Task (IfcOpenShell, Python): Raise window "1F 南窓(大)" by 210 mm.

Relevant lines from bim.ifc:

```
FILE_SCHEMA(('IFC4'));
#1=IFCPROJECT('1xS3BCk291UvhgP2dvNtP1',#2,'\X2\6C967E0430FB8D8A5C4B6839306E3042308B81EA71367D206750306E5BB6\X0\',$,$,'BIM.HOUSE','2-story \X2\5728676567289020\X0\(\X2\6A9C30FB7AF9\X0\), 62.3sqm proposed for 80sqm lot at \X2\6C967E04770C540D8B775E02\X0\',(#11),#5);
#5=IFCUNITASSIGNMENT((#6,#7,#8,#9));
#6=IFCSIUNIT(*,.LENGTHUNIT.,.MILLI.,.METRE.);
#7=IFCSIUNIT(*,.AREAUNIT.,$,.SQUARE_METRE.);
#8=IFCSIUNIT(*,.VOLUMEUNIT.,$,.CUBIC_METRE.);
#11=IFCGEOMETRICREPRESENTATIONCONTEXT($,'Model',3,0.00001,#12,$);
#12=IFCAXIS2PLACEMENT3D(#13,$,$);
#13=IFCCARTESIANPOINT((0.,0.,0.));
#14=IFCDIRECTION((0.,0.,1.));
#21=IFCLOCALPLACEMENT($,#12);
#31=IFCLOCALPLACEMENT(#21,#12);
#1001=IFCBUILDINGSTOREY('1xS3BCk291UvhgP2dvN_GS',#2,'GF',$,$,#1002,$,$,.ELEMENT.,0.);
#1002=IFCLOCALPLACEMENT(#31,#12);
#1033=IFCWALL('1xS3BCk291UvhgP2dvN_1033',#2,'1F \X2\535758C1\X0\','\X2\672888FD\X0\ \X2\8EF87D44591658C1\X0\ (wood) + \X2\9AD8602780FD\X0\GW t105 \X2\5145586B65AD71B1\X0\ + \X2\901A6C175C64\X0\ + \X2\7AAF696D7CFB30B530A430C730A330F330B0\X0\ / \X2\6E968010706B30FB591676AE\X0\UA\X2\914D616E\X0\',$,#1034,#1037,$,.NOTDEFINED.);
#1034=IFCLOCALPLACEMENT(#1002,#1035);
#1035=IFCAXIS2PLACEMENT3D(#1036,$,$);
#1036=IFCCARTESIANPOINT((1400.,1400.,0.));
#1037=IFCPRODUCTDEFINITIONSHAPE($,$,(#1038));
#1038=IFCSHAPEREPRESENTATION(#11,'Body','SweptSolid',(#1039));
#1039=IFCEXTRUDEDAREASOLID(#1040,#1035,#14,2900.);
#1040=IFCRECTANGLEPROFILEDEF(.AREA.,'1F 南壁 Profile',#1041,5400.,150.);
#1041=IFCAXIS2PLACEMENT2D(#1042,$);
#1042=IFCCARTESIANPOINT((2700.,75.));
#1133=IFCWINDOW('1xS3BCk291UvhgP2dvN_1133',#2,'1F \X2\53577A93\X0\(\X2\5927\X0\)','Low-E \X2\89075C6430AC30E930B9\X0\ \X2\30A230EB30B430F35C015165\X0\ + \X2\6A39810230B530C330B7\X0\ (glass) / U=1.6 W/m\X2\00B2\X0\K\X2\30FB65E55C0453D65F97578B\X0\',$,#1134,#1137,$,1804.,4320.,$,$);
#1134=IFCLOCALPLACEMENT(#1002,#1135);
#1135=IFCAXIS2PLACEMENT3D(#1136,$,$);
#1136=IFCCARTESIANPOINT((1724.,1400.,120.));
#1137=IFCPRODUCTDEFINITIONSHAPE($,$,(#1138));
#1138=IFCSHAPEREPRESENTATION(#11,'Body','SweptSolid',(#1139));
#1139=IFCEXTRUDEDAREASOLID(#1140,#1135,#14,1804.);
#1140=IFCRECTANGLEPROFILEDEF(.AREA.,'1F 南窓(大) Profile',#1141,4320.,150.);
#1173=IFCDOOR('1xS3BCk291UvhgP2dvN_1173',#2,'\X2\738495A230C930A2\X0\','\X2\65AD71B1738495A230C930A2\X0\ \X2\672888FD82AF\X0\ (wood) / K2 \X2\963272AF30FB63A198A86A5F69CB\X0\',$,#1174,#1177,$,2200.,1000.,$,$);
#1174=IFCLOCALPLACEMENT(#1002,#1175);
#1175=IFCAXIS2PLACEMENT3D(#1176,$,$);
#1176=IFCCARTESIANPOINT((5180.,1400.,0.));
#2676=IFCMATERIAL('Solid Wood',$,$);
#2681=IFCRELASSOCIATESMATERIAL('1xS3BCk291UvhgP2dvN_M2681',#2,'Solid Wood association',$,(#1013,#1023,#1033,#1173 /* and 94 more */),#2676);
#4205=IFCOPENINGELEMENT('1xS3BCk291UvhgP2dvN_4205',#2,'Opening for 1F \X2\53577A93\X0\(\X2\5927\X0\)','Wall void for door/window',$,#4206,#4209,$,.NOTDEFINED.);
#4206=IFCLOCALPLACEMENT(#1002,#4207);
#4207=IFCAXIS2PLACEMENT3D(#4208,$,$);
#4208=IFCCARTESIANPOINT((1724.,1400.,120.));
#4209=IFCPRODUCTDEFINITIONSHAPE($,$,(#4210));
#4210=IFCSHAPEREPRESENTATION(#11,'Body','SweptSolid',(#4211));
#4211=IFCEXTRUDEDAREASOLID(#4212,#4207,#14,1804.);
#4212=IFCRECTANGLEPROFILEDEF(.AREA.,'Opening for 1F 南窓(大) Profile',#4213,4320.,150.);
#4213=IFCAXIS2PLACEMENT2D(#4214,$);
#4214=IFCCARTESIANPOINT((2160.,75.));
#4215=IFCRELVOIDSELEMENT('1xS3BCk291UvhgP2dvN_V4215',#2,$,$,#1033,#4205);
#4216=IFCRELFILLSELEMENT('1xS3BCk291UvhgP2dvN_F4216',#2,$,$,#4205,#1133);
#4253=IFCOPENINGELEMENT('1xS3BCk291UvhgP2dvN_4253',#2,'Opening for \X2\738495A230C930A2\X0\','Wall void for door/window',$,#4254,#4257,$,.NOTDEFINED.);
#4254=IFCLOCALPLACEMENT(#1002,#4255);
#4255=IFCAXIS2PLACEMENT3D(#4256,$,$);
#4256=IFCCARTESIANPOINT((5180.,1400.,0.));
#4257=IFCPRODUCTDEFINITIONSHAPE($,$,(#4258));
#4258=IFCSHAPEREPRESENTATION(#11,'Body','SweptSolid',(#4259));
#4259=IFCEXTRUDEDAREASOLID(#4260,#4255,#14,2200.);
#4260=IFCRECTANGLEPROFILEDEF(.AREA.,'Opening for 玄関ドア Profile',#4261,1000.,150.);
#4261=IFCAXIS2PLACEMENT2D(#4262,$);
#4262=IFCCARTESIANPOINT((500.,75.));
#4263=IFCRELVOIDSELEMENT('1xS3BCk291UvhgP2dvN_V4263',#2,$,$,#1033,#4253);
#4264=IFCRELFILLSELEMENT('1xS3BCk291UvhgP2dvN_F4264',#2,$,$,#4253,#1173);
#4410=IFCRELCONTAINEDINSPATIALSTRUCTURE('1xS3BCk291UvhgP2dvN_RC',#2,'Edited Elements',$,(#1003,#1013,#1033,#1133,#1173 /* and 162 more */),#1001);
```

```python
import numpy as np
import ifcopenshell
import ifcopenshell.api.geometry
import ifcopenshell.util.placement
import ifcopenshell.util.unit

model = ifcopenshell.open("bim.ifc")
unit_scale = ifcopenshell.util.unit.calculate_unit_scale(model)

window = model.by_guid("1xS3BCk291UvhgP2dvN_1133")
opening = window.FillsVoids[0].RelatingOpeningElement
dz = 0.21 / unit_scale

shift = np.array([0.0, 0.0, dz])
# The window is not placed relative to its opening, so move both.
for product in (opening, window):
    matrix = ifcopenshell.util.placement.get_local_placement(product.ObjectPlacement)
    matrix[:3, 3] += shift
    ifcopenshell.api.geometry.edit_object_placement(model, product=product, matrix=matrix, is_si=False)

print(f"moved by {dz * unit_scale:+.3f} m")

model.write("bim_edited.ifc")
```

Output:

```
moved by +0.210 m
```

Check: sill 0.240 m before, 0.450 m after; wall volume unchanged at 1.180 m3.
